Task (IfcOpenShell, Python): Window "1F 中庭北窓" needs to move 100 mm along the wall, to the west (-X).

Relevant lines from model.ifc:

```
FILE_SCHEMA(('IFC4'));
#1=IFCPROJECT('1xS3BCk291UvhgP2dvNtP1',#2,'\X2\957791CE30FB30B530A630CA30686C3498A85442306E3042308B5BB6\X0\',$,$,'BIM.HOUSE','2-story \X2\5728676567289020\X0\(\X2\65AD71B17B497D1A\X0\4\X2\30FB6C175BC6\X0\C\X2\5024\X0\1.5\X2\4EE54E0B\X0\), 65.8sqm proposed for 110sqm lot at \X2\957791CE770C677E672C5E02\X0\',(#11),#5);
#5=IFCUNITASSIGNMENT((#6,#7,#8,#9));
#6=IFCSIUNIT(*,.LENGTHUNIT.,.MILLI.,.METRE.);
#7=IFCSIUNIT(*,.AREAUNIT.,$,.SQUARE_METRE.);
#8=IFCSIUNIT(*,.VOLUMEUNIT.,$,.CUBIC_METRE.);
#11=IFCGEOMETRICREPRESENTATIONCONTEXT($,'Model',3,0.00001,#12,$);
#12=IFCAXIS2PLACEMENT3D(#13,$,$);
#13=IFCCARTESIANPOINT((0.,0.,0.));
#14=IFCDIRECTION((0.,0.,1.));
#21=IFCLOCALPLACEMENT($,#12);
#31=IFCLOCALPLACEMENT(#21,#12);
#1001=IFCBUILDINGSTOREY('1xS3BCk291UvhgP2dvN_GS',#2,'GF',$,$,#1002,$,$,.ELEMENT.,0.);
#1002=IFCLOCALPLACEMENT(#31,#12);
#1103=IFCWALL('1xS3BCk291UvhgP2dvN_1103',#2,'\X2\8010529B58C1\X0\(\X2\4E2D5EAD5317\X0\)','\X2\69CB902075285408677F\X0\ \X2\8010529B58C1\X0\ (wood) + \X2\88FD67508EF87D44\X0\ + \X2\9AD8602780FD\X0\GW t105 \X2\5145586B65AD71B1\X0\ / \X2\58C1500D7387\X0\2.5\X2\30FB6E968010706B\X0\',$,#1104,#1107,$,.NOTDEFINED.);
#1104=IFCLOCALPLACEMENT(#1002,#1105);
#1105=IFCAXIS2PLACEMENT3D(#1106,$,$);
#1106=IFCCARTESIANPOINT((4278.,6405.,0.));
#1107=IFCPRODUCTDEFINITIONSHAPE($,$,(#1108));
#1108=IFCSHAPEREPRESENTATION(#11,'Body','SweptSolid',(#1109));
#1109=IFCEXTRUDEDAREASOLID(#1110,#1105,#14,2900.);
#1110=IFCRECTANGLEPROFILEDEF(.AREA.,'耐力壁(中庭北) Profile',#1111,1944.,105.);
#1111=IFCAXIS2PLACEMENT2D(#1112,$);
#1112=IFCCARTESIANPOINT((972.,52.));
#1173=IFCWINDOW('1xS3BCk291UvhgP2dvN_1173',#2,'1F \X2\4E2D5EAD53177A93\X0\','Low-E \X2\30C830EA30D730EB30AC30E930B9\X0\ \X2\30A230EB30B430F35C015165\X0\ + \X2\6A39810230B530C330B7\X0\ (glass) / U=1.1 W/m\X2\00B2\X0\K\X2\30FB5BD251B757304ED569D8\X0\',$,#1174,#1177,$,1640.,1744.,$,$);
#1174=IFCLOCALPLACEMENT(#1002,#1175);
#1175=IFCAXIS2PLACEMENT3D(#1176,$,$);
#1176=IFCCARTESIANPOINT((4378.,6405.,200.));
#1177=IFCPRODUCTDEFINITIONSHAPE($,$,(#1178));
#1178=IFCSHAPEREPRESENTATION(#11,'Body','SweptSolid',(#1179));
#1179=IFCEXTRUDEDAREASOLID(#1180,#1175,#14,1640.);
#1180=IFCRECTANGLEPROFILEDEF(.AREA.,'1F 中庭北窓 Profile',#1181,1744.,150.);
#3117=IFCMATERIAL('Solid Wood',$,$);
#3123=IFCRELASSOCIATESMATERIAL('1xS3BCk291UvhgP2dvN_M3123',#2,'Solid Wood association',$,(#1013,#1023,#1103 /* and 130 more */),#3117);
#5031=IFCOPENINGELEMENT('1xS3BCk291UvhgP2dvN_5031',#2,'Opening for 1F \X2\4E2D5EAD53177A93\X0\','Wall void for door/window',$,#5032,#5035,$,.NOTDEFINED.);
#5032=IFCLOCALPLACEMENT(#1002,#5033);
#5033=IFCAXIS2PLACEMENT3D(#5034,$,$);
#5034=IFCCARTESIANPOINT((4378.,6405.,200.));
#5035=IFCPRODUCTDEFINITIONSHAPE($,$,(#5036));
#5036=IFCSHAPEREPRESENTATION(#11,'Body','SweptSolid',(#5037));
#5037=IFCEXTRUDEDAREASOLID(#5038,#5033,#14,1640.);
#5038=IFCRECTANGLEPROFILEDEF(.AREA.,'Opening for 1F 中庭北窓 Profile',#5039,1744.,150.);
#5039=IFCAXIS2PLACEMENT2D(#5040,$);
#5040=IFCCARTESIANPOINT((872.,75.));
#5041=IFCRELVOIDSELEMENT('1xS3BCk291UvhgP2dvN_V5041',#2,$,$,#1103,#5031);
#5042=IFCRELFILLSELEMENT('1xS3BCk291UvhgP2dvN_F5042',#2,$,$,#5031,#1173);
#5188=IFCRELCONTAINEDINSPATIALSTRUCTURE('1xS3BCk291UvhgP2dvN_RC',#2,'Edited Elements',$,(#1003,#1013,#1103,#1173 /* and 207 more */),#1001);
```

```python
import ifcopenshell
import ifcopenshell.api.geometry
import ifcopenshell.util.placement
import ifcopenshell.util.unit

model = ifcopenshell.open("model.ifc")
unit_scale = ifcopenshell.util.unit.calculate_unit_scale(model)

window = model.by_guid("1xS3BCk291UvhgP2dvN_1173")
opening = window.FillsVoids[0].RelatingOpeningElement
wall = opening.VoidsElements[0].RelatingBuildingElement

wall_matrix = ifcopenshell.util.placement.get_local_placement(wall.ObjectPlacement)
shift = wall_matrix[:3, 0] * -0.1 / unit_scale
before = ifcopenshell.util.placement.get_local_placement(window.ObjectPlacement)[:3, 3].copy()

# The window is not placed relative to its opening, so move both.
for product in (opening, window):
    matrix = ifcopenshell.util.placement.get_local_placement(product.ObjectPlacement)
    matrix[:3, 3] += shift
    ifcopenshell.api.geometry.edit_object_placement(model, product=product, matrix=matrix, is_si=False)

after = ifcopenshell.util.placement.get_local_placement(window.ObjectPlacement)[:3, 3]
print("window moved by", (after - before).round(3) + 0.0)

model.write("model_rev.ifc")
```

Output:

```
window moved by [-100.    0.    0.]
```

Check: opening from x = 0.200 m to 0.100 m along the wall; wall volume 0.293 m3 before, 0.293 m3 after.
